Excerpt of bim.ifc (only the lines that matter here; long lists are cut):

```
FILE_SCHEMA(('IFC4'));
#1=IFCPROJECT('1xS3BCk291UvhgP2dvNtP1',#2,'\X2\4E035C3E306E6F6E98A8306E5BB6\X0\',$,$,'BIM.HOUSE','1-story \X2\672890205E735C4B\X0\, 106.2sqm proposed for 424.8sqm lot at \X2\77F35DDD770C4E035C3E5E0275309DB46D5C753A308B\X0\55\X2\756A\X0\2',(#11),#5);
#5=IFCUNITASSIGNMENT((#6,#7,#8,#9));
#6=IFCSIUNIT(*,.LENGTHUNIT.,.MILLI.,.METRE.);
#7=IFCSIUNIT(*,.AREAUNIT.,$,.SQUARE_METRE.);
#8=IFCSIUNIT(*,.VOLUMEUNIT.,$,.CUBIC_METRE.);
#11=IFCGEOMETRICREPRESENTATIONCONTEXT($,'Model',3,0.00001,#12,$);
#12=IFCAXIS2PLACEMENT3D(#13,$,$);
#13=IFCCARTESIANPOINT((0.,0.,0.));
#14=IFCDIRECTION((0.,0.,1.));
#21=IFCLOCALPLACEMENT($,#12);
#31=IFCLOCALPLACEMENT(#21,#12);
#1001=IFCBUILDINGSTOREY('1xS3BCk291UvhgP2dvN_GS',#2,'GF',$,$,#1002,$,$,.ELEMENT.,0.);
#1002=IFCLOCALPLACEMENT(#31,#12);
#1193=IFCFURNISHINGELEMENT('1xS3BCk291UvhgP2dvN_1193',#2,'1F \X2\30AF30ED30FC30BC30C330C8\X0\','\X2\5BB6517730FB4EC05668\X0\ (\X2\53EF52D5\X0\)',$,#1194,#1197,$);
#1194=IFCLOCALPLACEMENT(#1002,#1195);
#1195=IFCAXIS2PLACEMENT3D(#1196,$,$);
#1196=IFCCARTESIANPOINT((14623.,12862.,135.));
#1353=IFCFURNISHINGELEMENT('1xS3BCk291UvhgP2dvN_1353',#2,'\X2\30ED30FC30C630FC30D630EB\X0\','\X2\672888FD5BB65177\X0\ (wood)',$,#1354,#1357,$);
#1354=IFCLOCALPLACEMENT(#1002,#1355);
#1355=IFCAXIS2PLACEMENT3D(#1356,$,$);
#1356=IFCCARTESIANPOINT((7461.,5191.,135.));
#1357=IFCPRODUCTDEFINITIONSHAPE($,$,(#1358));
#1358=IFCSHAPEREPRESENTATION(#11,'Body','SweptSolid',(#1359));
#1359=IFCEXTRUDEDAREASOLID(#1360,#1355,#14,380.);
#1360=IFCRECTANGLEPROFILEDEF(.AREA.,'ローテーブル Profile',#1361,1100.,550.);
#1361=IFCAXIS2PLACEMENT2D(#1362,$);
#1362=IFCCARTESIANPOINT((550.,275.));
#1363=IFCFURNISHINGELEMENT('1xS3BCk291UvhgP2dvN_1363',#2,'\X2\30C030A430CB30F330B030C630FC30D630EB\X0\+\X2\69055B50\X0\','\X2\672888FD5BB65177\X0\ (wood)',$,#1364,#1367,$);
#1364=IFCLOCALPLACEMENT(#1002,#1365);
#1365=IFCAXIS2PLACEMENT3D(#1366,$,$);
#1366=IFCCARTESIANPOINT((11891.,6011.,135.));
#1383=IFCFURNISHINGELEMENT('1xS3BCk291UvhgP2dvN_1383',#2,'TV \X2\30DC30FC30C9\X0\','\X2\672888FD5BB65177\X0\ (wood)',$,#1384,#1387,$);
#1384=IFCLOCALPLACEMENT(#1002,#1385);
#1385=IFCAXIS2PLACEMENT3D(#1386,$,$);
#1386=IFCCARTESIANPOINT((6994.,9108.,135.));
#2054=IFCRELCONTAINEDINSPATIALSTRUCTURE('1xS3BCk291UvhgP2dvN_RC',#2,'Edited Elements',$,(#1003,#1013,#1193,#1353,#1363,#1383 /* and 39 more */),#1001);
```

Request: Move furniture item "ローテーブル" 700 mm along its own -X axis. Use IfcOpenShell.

```python
import ifcopenshell
import ifcopenshell.api.geometry
import ifcopenshell.util.placement

model = ifcopenshell.open("bim.ifc")

item = model.by_guid("1xS3BCk291UvhgP2dvN_1353")
matrix = ifcopenshell.util.placement.get_local_placement(item.ObjectPlacement)
matrix[:3, 3] -= matrix[:3, 0] * 700.0
ifcopenshell.api.geometry.edit_object_placement(model, product=item, matrix=matrix, is_si=False)

print(ifcopenshell.util.placement.get_local_placement(item.ObjectPlacement).round(3) + 0.0)

model.write("bim_edited.ifc")
```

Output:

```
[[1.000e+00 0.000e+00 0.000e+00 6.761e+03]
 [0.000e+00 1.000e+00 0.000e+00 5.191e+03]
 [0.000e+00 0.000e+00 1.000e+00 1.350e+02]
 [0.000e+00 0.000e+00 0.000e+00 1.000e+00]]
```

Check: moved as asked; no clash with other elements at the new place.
